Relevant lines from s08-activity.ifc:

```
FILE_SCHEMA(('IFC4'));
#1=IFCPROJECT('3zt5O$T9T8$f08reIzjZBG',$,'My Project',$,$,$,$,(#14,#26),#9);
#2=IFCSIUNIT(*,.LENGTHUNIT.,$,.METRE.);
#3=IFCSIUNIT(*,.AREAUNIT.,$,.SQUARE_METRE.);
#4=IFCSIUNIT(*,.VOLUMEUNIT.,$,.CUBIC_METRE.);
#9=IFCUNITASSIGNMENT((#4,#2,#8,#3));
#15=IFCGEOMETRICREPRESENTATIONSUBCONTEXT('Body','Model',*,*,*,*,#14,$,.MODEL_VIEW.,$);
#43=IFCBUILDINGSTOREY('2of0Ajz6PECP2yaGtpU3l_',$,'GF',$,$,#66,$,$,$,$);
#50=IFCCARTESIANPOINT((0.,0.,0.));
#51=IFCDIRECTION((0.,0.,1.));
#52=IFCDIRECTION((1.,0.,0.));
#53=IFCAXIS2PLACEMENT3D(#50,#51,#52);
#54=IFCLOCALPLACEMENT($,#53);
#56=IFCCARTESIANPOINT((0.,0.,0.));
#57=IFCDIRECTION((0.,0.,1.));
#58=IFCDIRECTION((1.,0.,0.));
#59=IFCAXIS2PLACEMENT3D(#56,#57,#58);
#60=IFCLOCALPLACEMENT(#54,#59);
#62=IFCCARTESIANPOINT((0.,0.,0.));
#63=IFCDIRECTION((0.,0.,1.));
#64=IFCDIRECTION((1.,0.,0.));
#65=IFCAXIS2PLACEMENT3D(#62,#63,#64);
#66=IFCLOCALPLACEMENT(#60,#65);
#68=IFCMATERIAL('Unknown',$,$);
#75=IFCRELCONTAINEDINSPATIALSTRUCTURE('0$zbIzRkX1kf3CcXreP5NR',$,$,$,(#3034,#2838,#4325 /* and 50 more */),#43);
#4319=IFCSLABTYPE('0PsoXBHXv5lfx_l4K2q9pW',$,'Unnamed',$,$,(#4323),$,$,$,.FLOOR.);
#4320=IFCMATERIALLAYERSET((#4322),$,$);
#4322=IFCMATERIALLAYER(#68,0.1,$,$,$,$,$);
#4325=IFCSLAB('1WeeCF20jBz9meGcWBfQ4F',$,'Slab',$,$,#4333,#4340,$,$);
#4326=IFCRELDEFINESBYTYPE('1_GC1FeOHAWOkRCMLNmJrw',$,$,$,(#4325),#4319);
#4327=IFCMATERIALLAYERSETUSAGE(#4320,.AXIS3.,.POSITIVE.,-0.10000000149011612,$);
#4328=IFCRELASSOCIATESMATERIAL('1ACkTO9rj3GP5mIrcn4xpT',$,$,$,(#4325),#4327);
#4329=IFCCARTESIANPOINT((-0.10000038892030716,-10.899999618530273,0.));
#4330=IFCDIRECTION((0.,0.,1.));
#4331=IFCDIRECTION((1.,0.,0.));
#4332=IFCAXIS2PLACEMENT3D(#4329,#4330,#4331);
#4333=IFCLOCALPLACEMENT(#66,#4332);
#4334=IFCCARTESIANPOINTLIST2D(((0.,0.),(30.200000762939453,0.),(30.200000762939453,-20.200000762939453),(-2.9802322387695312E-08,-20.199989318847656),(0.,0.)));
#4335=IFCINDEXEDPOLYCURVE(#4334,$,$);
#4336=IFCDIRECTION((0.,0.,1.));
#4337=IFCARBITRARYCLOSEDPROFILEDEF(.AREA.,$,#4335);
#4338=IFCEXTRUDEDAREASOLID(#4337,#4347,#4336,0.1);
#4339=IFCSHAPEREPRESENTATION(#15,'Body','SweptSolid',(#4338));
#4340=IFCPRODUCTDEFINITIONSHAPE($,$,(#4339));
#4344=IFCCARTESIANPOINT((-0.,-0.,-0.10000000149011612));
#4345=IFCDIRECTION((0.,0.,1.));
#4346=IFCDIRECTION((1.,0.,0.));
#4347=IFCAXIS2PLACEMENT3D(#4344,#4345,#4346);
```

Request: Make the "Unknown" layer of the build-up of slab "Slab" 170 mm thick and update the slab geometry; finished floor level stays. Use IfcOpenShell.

```python
import ifcopenshell
import ifcopenshell.util.element
import ifcopenshell.util.representation
import ifcopenshell.util.unit

model = ifcopenshell.open("s08-activity.ifc")
unit_scale = ifcopenshell.util.unit.calculate_unit_scale(model)

layer_set = model.by_id(4320)
layer = next(l for l in layer_set.MaterialLayers if l.Material and l.Material.Name == "Unknown")
change = 0.17 / unit_scale - layer.LayerThickness
layer.LayerThickness += change

# Geometry does not follow the layer set by itself.
slabs = [e for e in ifcopenshell.util.element.get_elements_by_material(model, layer_set) if e.is_a("IfcSlab")]
for slab in sorted(slabs, key=lambda e: e.id()):
    body = ifcopenshell.util.representation.get_representation(slab, "Model", "Body")
    solid = body.Items[0]
    old_depth = solid.Depth
    solid.Depth += change
    # Extruded upwards: lower the start of the extrusion so the top stays.
    x, y, z = solid.Position.Location.Coordinates
    solid.Position.Location = model.createIfcCartesianPoint((x, y, z - change))
    print(slab.id(), f"{old_depth:g} -> {solid.Depth:g}")

# The layers are counted up from the underside, which has moved.
for usage in {ifcopenshell.util.element.get_material(slab) for slab in slabs}:
    usage.OffsetFromReferenceLine -= change

model.write("s08-activity_v2.ifc")
```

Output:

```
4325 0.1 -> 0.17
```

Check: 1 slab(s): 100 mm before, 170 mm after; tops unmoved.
